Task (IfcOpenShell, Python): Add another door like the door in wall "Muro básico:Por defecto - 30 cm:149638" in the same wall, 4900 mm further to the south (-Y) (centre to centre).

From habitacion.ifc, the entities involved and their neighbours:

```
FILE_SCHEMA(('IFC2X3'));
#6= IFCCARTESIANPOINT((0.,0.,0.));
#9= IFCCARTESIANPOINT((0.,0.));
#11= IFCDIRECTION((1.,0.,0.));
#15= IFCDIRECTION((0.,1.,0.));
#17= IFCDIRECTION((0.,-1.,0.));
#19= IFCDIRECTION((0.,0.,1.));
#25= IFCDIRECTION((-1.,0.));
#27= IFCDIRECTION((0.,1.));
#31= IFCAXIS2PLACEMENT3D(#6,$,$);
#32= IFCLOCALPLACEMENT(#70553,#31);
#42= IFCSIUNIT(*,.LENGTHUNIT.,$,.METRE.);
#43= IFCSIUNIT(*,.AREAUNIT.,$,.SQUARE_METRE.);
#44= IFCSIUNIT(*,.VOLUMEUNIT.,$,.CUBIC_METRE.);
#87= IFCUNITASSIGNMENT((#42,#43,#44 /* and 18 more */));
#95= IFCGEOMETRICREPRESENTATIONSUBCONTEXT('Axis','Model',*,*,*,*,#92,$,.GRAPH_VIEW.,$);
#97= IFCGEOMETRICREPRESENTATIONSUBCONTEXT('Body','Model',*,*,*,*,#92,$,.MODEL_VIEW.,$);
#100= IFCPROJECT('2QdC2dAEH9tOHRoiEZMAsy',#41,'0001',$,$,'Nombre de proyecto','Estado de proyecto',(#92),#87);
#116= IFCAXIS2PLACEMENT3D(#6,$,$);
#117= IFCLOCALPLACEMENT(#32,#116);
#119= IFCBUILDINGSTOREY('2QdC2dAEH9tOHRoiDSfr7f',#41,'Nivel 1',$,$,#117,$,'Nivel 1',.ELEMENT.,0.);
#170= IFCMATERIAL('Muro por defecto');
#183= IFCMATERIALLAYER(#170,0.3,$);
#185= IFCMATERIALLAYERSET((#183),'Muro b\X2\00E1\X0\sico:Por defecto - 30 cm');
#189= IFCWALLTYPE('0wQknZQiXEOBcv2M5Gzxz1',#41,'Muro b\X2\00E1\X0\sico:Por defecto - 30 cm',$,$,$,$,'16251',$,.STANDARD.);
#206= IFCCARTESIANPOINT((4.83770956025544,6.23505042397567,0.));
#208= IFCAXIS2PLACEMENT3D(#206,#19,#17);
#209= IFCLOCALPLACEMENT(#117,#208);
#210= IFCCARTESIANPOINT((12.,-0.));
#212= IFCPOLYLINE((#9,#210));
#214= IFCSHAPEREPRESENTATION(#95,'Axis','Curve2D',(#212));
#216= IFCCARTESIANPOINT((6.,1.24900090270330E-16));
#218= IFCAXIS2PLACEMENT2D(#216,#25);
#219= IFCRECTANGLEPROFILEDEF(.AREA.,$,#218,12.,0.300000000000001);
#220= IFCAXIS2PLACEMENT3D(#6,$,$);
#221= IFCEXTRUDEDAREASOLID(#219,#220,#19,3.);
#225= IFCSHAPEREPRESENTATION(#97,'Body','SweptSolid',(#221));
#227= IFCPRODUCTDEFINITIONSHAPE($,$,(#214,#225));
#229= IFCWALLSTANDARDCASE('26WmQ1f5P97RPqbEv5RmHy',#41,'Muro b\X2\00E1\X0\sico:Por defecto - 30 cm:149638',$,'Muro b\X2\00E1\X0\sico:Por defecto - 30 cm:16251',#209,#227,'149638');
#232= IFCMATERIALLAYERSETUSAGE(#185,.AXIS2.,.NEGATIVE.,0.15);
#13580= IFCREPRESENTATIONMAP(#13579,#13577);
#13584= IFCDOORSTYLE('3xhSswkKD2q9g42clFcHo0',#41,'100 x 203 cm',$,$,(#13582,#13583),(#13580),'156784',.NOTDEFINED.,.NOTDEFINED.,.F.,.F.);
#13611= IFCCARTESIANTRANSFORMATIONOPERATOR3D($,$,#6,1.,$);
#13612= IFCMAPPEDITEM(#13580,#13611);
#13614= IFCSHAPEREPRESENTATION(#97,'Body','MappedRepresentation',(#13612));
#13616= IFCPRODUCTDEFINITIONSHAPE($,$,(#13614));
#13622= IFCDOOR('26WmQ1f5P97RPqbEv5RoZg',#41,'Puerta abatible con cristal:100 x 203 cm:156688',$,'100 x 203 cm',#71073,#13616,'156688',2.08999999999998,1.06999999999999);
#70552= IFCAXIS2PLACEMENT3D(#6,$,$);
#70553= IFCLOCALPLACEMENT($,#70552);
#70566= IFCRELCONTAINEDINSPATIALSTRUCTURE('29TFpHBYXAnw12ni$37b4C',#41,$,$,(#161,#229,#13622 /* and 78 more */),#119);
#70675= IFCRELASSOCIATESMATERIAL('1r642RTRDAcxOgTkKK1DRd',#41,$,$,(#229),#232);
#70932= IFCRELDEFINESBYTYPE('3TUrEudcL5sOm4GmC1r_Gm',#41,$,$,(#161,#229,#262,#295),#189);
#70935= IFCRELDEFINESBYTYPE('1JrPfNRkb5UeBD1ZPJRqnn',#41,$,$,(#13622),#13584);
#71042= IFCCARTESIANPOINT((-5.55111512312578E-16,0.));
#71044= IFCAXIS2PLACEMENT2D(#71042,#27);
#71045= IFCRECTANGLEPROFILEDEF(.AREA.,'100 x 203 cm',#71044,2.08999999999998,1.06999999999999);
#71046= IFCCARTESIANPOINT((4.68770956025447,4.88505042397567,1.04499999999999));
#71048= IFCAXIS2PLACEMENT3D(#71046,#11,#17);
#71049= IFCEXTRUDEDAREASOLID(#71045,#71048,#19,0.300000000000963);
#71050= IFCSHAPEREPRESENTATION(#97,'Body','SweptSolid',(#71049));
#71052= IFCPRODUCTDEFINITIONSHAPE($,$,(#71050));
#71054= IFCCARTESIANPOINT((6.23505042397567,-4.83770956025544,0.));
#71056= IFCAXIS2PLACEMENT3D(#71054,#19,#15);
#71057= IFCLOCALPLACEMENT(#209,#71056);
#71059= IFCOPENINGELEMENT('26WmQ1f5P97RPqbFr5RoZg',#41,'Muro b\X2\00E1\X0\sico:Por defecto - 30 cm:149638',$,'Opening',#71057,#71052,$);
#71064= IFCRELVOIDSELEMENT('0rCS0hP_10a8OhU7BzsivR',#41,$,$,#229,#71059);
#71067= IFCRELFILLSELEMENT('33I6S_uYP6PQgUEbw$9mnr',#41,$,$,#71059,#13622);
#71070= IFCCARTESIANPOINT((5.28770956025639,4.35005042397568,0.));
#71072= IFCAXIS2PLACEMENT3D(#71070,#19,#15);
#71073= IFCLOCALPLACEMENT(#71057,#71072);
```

```python
import ifcopenshell
import ifcopenshell.api.feature
import ifcopenshell.api.geometry
import ifcopenshell.api.root
import ifcopenshell.geom
import ifcopenshell.util.element
import ifcopenshell.util.placement
import ifcopenshell.util.shape
import ifcopenshell.util.unit

model = ifcopenshell.open("habitacion.ifc")
unit_scale = ifcopenshell.util.unit.calculate_unit_scale(model)
settings = ifcopenshell.geom.settings()


def volume(element):
    """Net volume in cubic metres, openings subtracted."""
    shape = ifcopenshell.geom.create_shape(settings, element)
    return ifcopenshell.util.shape.get_volume(shape.geometry)


def reuse_history(source, copy):
    """copy_class also copies each property set's owner history, people and application; keep the originals."""
    for rel in copy.IsDefinedBy:
        if rel.is_a("IfcRelDefinesByProperties") and (history := rel.RelatingPropertyDefinition.OwnerHistory):
            rel.RelatingPropertyDefinition.OwnerHistory = source.OwnerHistory
            ifcopenshell.util.element.remove_deep2(model, history)


door = model.by_guid("26WmQ1f5P97RPqbEv5RoZg")
opening = door.FillsVoids[0].RelatingOpeningElement
wall = opening.VoidsElements[0].RelatingBuildingElement
before = volume(wall)
shift = ifcopenshell.util.placement.get_local_placement(wall.ObjectPlacement)[:3, 0] * 4.9 / unit_scale

# copy_class copies the void relationship, type, container and properties, but no geometry.
new_opening = ifcopenshell.api.root.copy_class(model, product=opening)
new_opening.Representation = ifcopenshell.util.element.copy_deep(
    model, opening.Representation, exclude=["IfcGeometricRepresentationContext", "IfcRepresentationMap"]
)
new_opening.Name = "Muro básico:Por defecto - 30 cm"
new_door = ifcopenshell.api.root.copy_class(model, product=door)
new_door.Representation = ifcopenshell.util.element.copy_deep(
    model, door.Representation, exclude=["IfcGeometricRepresentationContext", "IfcRepresentationMap"]
)
new_door.Name = "Puerta abatible con cristal:100 x 203 cm"
new_door.Tag = None
reuse_history(door, new_door)
fills = ifcopenshell.api.feature.add_filling(model, opening=new_opening, element=new_door)
fills.OwnerHistory = new_door.OwnerHistory  # required in IFC2X3

for old, new in ((opening, new_opening), (door, new_door)):
    matrix = ifcopenshell.util.placement.get_local_placement(old.ObjectPlacement)
    matrix[:3, 3] += shift
    ifcopenshell.api.geometry.edit_object_placement(model, product=new, matrix=matrix, is_si=False)

after = volume(wall)

print(f"wall volume {before:.3f} -> {after:.3f} m3")

model.write("habitacion-out.ifc")
```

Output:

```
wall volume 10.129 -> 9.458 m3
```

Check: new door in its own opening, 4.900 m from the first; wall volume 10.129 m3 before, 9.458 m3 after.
